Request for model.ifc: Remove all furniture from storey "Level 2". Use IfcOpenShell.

First a look at what the model holds.

```python
import ifcopenshell
import ifcopenshell.util.element

model = ifcopenshell.open("model.ifc")
print(model.schema)
storey = next(s for s in model.by_type("IfcBuildingStorey") if s.Name == "Level 2")
furniture = [e for e in ifcopenshell.util.element.get_decomposition(storey) if e.is_a("IfcFurnishingElement")]
seen = {}
for e in furniture:
    element_type = ifcopenshell.util.element.get_type(e)
    name = element_type.Name if element_type not in (None, e) else None
    seen[name] = seen.get(name, 0) + 1
for name, count in sorted(seen.items(), key=str):
    print(count, "x", name)
```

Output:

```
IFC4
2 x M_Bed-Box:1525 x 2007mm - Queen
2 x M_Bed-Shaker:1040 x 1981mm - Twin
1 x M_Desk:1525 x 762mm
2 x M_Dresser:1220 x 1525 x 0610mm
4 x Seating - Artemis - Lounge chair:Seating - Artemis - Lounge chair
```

```python
import ifcopenshell
import ifcopenshell.api.root
import ifcopenshell.util.element

model = ifcopenshell.open("model.ifc")

storey = next(s for s in model.by_type("IfcBuildingStorey") if s.Name == "Level 2")
furniture = [e for e in ifcopenshell.util.element.get_decomposition(storey) if e.is_a("IfcFurnishingElement")]

for e in furniture:
    ifcopenshell.api.root.remove_product(model, product=e)
print(len(furniture), "removed")

model.write("model_rev.ifc")
```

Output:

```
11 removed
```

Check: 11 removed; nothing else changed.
